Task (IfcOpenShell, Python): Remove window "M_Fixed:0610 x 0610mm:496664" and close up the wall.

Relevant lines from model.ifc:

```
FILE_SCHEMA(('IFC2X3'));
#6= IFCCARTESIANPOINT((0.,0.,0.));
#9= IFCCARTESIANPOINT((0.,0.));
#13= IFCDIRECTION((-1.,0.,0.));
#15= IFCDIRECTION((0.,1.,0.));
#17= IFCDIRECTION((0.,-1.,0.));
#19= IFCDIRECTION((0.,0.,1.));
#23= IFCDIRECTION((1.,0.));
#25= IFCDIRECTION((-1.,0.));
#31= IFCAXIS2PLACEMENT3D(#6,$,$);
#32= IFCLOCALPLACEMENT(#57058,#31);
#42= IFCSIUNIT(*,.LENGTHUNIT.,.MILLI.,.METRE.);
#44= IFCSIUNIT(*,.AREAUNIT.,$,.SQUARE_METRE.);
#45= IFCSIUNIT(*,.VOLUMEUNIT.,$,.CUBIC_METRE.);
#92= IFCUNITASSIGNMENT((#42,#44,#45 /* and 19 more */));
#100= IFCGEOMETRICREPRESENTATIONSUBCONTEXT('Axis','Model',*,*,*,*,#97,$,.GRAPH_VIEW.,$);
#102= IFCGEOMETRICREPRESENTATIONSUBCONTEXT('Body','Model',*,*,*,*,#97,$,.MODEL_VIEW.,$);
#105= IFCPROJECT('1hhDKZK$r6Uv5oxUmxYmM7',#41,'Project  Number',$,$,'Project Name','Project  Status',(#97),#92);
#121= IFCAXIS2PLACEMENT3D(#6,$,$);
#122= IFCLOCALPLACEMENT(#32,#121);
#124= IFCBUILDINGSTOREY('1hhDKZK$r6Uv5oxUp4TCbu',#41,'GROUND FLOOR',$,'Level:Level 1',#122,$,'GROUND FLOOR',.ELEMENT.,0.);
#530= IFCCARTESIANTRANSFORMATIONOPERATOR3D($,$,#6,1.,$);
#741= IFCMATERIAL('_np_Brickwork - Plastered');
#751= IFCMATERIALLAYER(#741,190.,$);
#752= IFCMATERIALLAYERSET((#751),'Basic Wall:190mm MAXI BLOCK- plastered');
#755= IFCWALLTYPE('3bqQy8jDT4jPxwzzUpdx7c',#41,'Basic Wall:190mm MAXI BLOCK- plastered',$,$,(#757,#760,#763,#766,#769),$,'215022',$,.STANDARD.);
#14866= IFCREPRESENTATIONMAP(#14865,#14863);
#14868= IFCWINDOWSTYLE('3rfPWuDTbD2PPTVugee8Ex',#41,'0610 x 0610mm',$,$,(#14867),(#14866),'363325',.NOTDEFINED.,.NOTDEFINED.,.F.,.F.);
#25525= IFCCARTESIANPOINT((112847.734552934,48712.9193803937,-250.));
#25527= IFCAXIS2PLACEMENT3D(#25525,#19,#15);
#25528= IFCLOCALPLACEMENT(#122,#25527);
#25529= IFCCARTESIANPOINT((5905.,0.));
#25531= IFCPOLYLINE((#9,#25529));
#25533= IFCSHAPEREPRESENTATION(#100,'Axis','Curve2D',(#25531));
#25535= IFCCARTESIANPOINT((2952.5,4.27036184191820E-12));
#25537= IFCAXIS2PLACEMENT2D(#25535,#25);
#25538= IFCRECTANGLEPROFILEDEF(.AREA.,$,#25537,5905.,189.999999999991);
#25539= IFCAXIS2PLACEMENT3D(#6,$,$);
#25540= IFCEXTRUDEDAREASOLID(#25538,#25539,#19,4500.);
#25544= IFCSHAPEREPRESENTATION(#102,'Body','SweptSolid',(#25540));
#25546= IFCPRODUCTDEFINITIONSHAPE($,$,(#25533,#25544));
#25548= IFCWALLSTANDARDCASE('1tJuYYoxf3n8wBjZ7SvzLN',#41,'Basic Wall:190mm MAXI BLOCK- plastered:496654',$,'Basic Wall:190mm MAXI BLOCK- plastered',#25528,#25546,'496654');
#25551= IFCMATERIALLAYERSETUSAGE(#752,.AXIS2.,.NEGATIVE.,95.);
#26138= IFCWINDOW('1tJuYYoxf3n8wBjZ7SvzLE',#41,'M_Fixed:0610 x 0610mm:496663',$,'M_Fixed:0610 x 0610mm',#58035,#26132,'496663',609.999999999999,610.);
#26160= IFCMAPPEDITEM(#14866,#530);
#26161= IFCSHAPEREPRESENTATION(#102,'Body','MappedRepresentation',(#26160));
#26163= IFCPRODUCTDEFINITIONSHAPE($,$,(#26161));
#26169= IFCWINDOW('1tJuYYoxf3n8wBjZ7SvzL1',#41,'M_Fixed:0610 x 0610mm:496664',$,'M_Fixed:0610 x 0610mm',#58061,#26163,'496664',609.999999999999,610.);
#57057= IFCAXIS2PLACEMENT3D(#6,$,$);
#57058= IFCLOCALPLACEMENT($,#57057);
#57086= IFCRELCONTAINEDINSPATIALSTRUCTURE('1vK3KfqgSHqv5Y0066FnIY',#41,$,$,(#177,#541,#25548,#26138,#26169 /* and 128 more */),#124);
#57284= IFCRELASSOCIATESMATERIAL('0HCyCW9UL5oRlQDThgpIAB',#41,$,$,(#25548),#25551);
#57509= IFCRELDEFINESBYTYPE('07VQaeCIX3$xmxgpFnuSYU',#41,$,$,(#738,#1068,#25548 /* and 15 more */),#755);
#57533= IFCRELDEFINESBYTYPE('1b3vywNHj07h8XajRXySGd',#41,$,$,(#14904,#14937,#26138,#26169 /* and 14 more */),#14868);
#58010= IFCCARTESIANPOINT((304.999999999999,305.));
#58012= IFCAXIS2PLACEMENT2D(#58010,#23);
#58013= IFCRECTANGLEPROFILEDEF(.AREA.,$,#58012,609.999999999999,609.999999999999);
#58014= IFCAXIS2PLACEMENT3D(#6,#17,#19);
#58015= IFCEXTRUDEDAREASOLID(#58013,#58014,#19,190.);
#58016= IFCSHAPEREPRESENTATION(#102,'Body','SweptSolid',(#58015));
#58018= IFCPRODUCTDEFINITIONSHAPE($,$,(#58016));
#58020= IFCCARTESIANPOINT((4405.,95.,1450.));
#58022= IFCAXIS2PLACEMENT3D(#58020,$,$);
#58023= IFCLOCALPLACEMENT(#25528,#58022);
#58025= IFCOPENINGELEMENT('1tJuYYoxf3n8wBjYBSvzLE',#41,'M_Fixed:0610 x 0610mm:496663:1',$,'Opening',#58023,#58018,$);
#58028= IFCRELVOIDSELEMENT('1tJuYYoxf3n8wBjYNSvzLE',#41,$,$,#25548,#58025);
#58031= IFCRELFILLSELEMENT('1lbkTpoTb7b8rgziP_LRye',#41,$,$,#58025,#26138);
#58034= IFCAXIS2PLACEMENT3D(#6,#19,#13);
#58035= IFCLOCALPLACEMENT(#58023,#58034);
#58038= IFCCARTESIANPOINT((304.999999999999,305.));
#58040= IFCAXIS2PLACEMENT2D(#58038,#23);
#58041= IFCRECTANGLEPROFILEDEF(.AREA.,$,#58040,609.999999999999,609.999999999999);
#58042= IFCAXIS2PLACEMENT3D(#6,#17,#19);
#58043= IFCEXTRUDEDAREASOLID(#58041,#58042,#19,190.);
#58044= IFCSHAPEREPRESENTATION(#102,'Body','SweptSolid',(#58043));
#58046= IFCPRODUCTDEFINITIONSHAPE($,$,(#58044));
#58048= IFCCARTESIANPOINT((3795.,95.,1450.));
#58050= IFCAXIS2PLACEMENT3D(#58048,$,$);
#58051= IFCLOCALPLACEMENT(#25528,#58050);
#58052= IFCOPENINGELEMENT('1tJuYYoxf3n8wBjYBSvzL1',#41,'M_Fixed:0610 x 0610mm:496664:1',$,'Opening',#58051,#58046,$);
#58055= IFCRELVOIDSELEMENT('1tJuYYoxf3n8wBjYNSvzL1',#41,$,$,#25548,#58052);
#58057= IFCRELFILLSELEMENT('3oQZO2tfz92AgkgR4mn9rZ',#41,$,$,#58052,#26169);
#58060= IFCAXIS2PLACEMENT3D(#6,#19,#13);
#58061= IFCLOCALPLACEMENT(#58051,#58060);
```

```python
import ifcopenshell
import ifcopenshell.api.feature
import ifcopenshell.api.root
import ifcopenshell.geom
import ifcopenshell.util.shape

model = ifcopenshell.open("model.ifc")
settings = ifcopenshell.geom.settings()


def volume(element):
    """Net volume in cubic metres, openings subtracted."""
    shape = ifcopenshell.geom.create_shape(settings, element)
    return ifcopenshell.util.shape.get_volume(shape.geometry)


window = model.by_guid("1tJuYYoxf3n8wBjZ7SvzL1")
opening = window.FillsVoids[0].RelatingOpeningElement
wall = opening.VoidsElements[0].RelatingBuildingElement
before = volume(wall)

ifcopenshell.api.root.remove_product(model, product=window)
ifcopenshell.api.feature.remove_feature(model, feature=opening)

after = volume(wall)

print(f"wall volume {before:.3f} -> {after:.3f} m3")

model.write("model_updated.ifc")
```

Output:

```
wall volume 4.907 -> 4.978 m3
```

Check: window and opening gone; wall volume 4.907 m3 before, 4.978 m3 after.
